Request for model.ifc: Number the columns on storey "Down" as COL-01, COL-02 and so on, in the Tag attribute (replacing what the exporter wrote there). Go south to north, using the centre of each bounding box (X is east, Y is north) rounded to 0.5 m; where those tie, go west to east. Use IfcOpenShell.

First a look at what the model holds.

```python
import ifcopenshell
import ifcopenshell.util.element
import ifcopenshell.util.placement

model = ifcopenshell.open("model.ifc")
print(model.schema)
storey = next(s for s in model.by_type("IfcBuildingStorey") if s.Name == "Down")
columns = [e for e in ifcopenshell.util.element.get_decomposition(storey) if e.is_a("IfcColumn")]
for e in sorted(columns, key=lambda e: e.id()):
    origin = ifcopenshell.util.placement.get_local_placement(e.ObjectPlacement)[:3, 3]
    print(e.id(), e.Tag, e.Name, origin.round(2) + 0.0, sep=" | ")
```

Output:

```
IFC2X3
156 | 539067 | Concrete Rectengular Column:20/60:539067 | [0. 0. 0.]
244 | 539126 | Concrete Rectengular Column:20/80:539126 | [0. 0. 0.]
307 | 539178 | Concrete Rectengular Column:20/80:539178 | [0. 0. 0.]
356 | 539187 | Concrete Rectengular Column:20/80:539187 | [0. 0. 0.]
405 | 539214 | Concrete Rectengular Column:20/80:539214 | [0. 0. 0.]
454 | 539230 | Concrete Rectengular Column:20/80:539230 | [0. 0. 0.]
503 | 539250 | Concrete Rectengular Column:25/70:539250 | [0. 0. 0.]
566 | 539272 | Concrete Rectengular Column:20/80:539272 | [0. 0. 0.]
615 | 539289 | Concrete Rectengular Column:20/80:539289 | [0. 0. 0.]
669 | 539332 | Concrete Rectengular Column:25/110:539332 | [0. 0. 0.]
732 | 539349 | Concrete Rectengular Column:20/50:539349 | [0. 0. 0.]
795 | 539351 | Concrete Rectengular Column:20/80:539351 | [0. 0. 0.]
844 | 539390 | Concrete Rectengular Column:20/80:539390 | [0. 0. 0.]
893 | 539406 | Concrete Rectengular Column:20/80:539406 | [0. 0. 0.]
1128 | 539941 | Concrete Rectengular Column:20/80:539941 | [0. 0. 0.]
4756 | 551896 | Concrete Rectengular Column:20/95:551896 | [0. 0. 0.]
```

```python
import ifcopenshell
import ifcopenshell.geom
import ifcopenshell.util.element
import ifcopenshell.util.shape

model = ifcopenshell.open("model.ifc")
settings = ifcopenshell.geom.settings()
settings.set("use-world-coords", True)


def centre(element):
    shape = ifcopenshell.geom.create_shape(settings, element)
    return ifcopenshell.util.shape.get_bbox_centroid(shape.geometry)


storey = next(s for s in model.by_type("IfcBuildingStorey") if s.Name == "Down")
columns = [e for e in ifcopenshell.util.element.get_decomposition(storey) if e.is_a("IfcColumn")]

# Insertion points can sit at a corner or the storey origin, so sort by the geometry (in metres).
centres = {e: centre(e) for e in columns}
columns.sort(key=lambda e: (round(centres[e][1] / 0.5), centres[e][0]))

for i, e in enumerate(columns, start=1):
    number = f"COL-{i:02d}"
    e.Tag = number
    print(e.id(), number)

model.write("model_edited.ifc")
```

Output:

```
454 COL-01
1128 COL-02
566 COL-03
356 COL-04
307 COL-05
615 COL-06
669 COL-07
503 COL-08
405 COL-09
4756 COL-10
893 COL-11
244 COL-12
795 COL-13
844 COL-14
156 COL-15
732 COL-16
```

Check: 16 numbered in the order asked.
